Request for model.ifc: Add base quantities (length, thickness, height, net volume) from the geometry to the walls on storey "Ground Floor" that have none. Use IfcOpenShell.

First a look at what the model holds.

```python
import ifcopenshell
import ifcopenshell.util.element
import ifcopenshell.util.unit

model = ifcopenshell.open("model.ifc")
print(model.schema)
for unit_type in ("LENGTHUNIT", "AREAUNIT", "VOLUMEUNIT"):
    print(unit_type, ifcopenshell.util.unit.calculate_unit_scale(model, unit_type))
storey = next(s for s in model.by_type("IfcBuildingStorey") if s.Name == "Ground Floor")
walls = [e for e in ifcopenshell.util.element.get_decomposition(storey) if e.is_a("IfcWall")]
for e in sorted(walls, key=lambda e: e.id()):
    print(e.id(), e.is_a(), e.Name, list(ifcopenshell.util.element.get_psets(e, qtos_only=True)), sep=" | ")
```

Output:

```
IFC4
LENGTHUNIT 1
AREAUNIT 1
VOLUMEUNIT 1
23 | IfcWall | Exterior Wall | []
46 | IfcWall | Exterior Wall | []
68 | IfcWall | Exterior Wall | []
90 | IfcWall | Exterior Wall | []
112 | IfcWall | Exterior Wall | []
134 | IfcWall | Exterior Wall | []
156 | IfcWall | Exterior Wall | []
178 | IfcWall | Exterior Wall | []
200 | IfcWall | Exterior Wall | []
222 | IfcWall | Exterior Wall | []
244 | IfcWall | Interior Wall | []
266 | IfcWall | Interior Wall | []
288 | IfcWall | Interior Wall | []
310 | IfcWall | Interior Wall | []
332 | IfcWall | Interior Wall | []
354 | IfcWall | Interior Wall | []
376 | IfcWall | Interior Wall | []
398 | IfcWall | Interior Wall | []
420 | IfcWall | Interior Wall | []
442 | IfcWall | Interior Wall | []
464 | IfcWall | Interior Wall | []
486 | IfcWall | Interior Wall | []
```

```python
import ifcopenshell
import ifcopenshell.api.pset
import ifcopenshell.geom
import ifcopenshell.util.element
import ifcopenshell.util.shape
import ifcopenshell.util.unit

model = ifcopenshell.open("model.ifc")
unit_scale = ifcopenshell.util.unit.calculate_unit_scale(model)
volume_scale = ifcopenshell.util.unit.calculate_unit_scale(model, "VOLUMEUNIT")
settings = ifcopenshell.geom.settings()

storey = next(s for s in model.by_type("IfcBuildingStorey") if s.Name == "Ground Floor")
walls = [e for e in ifcopenshell.util.element.get_decomposition(storey) if e.is_a("IfcWall")]

for e in sorted(walls, key=lambda e: e.id()):
    if ifcopenshell.util.element.get_psets(e, qtos_only=True, should_inherit=False):
        continue
    # Geometry comes back in metres, in the element's own axes.
    shape = ifcopenshell.geom.create_shape(settings, e)
    values = {
        "Length": ifcopenshell.util.shape.get_x(shape.geometry) / unit_scale,
        "Width": ifcopenshell.util.shape.get_y(shape.geometry) / unit_scale,
        "Height": ifcopenshell.util.shape.get_z(shape.geometry) / unit_scale,
        "NetVolume": ifcopenshell.util.shape.get_volume(shape.geometry) / volume_scale,
    }
    qto = ifcopenshell.api.pset.add_qto(model, product=e, name="Qto_WallBaseQuantities")
    ifcopenshell.api.pset.edit_qto(model, qto=qto, properties=values)
    print(e.id(), {k: round(v, 3) for k, v in values.items()})

model.write("model_rev.ifc")
```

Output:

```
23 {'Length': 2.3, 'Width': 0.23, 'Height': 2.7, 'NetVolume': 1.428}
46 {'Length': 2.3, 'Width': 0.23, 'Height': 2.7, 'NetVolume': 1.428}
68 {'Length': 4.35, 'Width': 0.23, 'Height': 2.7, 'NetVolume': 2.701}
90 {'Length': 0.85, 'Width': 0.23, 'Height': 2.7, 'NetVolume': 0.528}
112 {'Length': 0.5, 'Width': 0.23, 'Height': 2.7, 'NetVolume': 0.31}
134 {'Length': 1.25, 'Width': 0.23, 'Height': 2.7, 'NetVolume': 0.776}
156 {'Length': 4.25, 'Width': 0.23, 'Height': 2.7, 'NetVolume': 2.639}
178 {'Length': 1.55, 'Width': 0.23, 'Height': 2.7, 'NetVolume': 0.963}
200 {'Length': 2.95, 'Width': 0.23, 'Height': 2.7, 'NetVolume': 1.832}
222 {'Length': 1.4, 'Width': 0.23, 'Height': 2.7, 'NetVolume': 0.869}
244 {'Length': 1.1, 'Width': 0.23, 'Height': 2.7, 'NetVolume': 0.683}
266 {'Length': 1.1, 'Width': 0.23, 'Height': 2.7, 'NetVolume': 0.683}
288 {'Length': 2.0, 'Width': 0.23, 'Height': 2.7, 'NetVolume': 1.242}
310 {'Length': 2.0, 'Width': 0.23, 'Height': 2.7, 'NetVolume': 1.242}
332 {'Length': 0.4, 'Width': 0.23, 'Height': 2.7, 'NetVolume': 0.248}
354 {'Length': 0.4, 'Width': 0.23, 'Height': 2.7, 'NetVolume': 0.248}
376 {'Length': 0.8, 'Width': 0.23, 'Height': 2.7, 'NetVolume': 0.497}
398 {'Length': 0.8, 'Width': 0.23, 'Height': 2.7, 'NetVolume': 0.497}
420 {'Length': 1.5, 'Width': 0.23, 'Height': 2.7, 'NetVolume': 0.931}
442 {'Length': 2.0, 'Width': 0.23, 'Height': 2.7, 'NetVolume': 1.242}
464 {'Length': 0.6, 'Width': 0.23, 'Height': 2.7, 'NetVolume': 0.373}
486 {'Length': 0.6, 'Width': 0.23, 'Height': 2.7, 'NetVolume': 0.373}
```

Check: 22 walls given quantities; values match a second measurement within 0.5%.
